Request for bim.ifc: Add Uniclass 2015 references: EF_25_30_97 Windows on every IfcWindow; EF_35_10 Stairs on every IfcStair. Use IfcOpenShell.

First a look at what the model holds.

```python
import ifcopenshell

model = ifcopenshell.open("bim.ifc")
print(model.schema)
print("classifications:", [c.Name for c in model.by_type("IfcClassification")])
for ifc_class in ("IfcDoor", "IfcRoof", "IfcStair", "IfcWall", "IfcWindow"):
    print(ifc_class, len(model.by_type(ifc_class)))
```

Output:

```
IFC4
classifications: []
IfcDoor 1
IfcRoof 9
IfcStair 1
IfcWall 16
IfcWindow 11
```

```python
import ifcopenshell
import ifcopenshell.api.classification

model = ifcopenshell.open("bim.ifc")

system = ifcopenshell.api.classification.add_classification(model, classification="Uniclass 2015")

codes = {
    "IfcWindow": ("EF_25_30_97", "Windows"),
    "IfcStair": ("EF_35_10", "Stairs"),
}
for ifc_class, (code, name) in codes.items():
    products = model.by_type(ifc_class)
    ifcopenshell.api.classification.add_reference(
        model, products=products, classification=system, identification=code, name=name
    )
    print(code, len(products))

model.write("bim_v2.ifc")
```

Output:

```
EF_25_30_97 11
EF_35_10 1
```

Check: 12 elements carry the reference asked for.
